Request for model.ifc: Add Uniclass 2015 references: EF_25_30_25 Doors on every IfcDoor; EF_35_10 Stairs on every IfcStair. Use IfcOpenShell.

First a look at what the model holds.

```python
import ifcopenshell

model = ifcopenshell.open("model.ifc")
print(model.schema)
print("classifications:", [c.Name for c in model.by_type("IfcClassification")])
for ifc_class in ("IfcDoor", "IfcRoof", "IfcStair", "IfcWall", "IfcWindow"):
    print(ifc_class, len(model.by_type(ifc_class)))
```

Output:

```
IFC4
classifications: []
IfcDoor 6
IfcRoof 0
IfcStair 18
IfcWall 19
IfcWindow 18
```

```python
import ifcopenshell
import ifcopenshell.api.classification

model = ifcopenshell.open("model.ifc")

system = ifcopenshell.api.classification.add_classification(model, classification="Uniclass 2015")

codes = {
    "IfcDoor": ("EF_25_30_25", "Doors"),
    "IfcStair": ("EF_35_10", "Stairs"),
}
for ifc_class, (code, name) in codes.items():
    products = model.by_type(ifc_class)
    ifcopenshell.api.classification.add_reference(
        model, products=products, classification=system, identification=code, name=name
    )
    print(code, len(products))

model.write("model_edited.ifc")
```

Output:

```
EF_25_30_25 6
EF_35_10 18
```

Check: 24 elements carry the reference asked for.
